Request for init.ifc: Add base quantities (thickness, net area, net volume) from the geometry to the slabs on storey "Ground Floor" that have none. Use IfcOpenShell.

First a look at what the model holds.

```python
import ifcopenshell
import ifcopenshell.util.element
import ifcopenshell.util.unit

model = ifcopenshell.open("init.ifc")
print(model.schema)
for unit_type in ("LENGTHUNIT", "AREAUNIT", "VOLUMEUNIT"):
    print(unit_type, ifcopenshell.util.unit.calculate_unit_scale(model, unit_type))
storey = next(s for s in model.by_type("IfcBuildingStorey") if s.Name == "Ground Floor")
slabs = [e for e in ifcopenshell.util.element.get_decomposition(storey) if e.is_a("IfcSlab")]
for e in sorted(slabs, key=lambda e: e.id()):
    print(e.id(), e.is_a(), e.Name, list(ifcopenshell.util.element.get_psets(e, qtos_only=True)), sep=" | ")
```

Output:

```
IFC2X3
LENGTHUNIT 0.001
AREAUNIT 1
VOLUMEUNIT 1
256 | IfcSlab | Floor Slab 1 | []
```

```python
import ifcopenshell
import ifcopenshell.api.pset
import ifcopenshell.geom
import ifcopenshell.util.element
import ifcopenshell.util.shape
import ifcopenshell.util.unit

model = ifcopenshell.open("init.ifc")
unit_scale = ifcopenshell.util.unit.calculate_unit_scale(model)
area_scale = ifcopenshell.util.unit.calculate_unit_scale(model, "AREAUNIT")
volume_scale = ifcopenshell.util.unit.calculate_unit_scale(model, "VOLUMEUNIT")
settings = ifcopenshell.geom.settings()

storey = next(s for s in model.by_type("IfcBuildingStorey") if s.Name == "Ground Floor")
slabs = [e for e in ifcopenshell.util.element.get_decomposition(storey) if e.is_a("IfcSlab")]

for e in sorted(slabs, key=lambda e: e.id()):
    if ifcopenshell.util.element.get_psets(e, qtos_only=True, should_inherit=False):
        continue
    # Geometry comes back in metres, in the element's own axes.
    shape = ifcopenshell.geom.create_shape(settings, e)
    values = {
        "Width": ifcopenshell.util.shape.get_z(shape.geometry) / unit_scale,
        "NetArea": ifcopenshell.util.shape.get_footprint_area(shape.geometry) / area_scale,
        "NetVolume": ifcopenshell.util.shape.get_volume(shape.geometry) / volume_scale,
    }
    qto = ifcopenshell.api.pset.add_qto(model, product=e, name="BaseQuantities")
    ifcopenshell.api.pset.edit_qto(model, qto=qto, properties=values)
    print(e.id(), {k: round(v, 3) for k, v in values.items()})

model.write("init_updated.ifc")
```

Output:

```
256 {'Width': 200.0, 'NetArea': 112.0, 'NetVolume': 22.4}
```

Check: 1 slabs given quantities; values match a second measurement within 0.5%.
